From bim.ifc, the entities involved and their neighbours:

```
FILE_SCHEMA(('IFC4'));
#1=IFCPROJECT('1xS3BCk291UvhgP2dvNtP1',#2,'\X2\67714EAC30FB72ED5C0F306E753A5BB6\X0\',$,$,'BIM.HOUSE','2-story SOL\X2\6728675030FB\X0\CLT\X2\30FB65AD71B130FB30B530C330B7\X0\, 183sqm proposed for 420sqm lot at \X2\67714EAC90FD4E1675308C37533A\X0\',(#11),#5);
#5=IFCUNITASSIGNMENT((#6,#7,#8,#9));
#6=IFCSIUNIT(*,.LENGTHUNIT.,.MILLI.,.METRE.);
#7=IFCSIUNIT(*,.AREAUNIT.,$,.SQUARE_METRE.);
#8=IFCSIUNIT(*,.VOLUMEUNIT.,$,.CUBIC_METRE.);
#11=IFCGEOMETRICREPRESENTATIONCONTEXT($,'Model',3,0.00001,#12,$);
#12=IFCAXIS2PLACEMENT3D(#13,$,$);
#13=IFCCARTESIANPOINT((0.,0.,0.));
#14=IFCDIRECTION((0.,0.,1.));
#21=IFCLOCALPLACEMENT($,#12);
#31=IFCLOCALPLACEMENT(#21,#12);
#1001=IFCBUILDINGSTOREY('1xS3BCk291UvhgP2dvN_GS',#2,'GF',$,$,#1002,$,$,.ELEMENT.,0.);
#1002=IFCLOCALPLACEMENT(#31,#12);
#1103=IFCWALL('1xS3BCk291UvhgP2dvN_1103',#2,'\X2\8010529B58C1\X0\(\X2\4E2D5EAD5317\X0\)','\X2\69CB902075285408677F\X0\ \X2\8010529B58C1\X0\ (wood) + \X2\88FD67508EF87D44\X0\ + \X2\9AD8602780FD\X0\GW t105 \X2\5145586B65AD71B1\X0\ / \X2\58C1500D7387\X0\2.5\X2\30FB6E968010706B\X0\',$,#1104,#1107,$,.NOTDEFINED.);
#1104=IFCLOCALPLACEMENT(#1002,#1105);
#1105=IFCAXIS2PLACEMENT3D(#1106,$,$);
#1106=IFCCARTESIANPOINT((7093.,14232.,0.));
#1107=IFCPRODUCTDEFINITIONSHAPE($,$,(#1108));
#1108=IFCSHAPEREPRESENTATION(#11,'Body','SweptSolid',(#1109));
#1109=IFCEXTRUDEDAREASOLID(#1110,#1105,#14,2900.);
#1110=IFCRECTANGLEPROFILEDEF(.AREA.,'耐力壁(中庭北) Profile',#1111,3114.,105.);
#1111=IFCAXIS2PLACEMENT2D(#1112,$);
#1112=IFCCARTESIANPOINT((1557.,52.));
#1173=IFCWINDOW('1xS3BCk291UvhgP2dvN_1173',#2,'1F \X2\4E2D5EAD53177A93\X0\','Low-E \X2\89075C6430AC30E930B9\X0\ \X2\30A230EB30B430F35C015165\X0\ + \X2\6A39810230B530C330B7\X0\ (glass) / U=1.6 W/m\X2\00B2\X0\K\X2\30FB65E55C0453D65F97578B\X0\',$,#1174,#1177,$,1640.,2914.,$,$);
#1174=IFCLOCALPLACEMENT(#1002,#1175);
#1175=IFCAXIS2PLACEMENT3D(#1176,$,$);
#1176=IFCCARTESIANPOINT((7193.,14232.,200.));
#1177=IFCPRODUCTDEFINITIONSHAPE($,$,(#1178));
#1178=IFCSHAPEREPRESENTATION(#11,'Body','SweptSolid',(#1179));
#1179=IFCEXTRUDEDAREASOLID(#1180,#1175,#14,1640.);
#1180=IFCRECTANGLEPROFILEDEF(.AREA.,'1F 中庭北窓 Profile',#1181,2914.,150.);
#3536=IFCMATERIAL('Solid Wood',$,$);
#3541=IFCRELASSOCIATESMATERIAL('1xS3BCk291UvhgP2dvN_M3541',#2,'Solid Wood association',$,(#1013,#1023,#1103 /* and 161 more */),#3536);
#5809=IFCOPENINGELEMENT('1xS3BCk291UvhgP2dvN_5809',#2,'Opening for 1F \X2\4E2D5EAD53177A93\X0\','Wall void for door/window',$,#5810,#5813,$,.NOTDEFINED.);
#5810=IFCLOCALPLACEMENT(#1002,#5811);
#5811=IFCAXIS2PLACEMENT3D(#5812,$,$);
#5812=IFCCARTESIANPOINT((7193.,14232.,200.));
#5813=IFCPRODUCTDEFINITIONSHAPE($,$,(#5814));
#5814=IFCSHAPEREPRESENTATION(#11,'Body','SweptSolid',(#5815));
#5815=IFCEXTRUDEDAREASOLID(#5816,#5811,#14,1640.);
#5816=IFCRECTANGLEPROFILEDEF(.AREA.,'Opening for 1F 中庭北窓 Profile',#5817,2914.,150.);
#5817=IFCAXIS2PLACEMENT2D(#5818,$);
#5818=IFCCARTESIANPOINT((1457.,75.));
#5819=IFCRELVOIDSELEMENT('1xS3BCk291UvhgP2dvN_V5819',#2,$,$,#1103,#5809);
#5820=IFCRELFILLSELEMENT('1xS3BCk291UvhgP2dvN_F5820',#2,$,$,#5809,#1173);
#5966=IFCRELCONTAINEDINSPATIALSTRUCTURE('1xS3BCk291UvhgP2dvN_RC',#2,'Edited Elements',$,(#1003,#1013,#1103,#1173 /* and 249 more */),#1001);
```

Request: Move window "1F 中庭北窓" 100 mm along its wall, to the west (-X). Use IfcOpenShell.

```python
import ifcopenshell
import ifcopenshell.api.geometry
import ifcopenshell.util.placement

model = ifcopenshell.open("bim.ifc")

window = model.by_guid("1xS3BCk291UvhgP2dvN_1173")
opening = window.FillsVoids[0].RelatingOpeningElement
wall = opening.VoidsElements[0].RelatingBuildingElement

wall_matrix = ifcopenshell.util.placement.get_local_placement(wall.ObjectPlacement)
shift = wall_matrix[:3, 0] * -100.0
before = ifcopenshell.util.placement.get_local_placement(window.ObjectPlacement)[:3, 3].copy()

# The window is not placed relative to its opening, so move both.
for product in (opening, window):
    matrix = ifcopenshell.util.placement.get_local_placement(product.ObjectPlacement)
    matrix[:3, 3] += shift
    ifcopenshell.api.geometry.edit_object_placement(model, product=product, matrix=matrix, is_si=False)

after = ifcopenshell.util.placement.get_local_placement(window.ObjectPlacement)[:3, 3]
print("window moved by", (after - before).round(3) + 0.0)

model.write("bim_updated.ifc")
```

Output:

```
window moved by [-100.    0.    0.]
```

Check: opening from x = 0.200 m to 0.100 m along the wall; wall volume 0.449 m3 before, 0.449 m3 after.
